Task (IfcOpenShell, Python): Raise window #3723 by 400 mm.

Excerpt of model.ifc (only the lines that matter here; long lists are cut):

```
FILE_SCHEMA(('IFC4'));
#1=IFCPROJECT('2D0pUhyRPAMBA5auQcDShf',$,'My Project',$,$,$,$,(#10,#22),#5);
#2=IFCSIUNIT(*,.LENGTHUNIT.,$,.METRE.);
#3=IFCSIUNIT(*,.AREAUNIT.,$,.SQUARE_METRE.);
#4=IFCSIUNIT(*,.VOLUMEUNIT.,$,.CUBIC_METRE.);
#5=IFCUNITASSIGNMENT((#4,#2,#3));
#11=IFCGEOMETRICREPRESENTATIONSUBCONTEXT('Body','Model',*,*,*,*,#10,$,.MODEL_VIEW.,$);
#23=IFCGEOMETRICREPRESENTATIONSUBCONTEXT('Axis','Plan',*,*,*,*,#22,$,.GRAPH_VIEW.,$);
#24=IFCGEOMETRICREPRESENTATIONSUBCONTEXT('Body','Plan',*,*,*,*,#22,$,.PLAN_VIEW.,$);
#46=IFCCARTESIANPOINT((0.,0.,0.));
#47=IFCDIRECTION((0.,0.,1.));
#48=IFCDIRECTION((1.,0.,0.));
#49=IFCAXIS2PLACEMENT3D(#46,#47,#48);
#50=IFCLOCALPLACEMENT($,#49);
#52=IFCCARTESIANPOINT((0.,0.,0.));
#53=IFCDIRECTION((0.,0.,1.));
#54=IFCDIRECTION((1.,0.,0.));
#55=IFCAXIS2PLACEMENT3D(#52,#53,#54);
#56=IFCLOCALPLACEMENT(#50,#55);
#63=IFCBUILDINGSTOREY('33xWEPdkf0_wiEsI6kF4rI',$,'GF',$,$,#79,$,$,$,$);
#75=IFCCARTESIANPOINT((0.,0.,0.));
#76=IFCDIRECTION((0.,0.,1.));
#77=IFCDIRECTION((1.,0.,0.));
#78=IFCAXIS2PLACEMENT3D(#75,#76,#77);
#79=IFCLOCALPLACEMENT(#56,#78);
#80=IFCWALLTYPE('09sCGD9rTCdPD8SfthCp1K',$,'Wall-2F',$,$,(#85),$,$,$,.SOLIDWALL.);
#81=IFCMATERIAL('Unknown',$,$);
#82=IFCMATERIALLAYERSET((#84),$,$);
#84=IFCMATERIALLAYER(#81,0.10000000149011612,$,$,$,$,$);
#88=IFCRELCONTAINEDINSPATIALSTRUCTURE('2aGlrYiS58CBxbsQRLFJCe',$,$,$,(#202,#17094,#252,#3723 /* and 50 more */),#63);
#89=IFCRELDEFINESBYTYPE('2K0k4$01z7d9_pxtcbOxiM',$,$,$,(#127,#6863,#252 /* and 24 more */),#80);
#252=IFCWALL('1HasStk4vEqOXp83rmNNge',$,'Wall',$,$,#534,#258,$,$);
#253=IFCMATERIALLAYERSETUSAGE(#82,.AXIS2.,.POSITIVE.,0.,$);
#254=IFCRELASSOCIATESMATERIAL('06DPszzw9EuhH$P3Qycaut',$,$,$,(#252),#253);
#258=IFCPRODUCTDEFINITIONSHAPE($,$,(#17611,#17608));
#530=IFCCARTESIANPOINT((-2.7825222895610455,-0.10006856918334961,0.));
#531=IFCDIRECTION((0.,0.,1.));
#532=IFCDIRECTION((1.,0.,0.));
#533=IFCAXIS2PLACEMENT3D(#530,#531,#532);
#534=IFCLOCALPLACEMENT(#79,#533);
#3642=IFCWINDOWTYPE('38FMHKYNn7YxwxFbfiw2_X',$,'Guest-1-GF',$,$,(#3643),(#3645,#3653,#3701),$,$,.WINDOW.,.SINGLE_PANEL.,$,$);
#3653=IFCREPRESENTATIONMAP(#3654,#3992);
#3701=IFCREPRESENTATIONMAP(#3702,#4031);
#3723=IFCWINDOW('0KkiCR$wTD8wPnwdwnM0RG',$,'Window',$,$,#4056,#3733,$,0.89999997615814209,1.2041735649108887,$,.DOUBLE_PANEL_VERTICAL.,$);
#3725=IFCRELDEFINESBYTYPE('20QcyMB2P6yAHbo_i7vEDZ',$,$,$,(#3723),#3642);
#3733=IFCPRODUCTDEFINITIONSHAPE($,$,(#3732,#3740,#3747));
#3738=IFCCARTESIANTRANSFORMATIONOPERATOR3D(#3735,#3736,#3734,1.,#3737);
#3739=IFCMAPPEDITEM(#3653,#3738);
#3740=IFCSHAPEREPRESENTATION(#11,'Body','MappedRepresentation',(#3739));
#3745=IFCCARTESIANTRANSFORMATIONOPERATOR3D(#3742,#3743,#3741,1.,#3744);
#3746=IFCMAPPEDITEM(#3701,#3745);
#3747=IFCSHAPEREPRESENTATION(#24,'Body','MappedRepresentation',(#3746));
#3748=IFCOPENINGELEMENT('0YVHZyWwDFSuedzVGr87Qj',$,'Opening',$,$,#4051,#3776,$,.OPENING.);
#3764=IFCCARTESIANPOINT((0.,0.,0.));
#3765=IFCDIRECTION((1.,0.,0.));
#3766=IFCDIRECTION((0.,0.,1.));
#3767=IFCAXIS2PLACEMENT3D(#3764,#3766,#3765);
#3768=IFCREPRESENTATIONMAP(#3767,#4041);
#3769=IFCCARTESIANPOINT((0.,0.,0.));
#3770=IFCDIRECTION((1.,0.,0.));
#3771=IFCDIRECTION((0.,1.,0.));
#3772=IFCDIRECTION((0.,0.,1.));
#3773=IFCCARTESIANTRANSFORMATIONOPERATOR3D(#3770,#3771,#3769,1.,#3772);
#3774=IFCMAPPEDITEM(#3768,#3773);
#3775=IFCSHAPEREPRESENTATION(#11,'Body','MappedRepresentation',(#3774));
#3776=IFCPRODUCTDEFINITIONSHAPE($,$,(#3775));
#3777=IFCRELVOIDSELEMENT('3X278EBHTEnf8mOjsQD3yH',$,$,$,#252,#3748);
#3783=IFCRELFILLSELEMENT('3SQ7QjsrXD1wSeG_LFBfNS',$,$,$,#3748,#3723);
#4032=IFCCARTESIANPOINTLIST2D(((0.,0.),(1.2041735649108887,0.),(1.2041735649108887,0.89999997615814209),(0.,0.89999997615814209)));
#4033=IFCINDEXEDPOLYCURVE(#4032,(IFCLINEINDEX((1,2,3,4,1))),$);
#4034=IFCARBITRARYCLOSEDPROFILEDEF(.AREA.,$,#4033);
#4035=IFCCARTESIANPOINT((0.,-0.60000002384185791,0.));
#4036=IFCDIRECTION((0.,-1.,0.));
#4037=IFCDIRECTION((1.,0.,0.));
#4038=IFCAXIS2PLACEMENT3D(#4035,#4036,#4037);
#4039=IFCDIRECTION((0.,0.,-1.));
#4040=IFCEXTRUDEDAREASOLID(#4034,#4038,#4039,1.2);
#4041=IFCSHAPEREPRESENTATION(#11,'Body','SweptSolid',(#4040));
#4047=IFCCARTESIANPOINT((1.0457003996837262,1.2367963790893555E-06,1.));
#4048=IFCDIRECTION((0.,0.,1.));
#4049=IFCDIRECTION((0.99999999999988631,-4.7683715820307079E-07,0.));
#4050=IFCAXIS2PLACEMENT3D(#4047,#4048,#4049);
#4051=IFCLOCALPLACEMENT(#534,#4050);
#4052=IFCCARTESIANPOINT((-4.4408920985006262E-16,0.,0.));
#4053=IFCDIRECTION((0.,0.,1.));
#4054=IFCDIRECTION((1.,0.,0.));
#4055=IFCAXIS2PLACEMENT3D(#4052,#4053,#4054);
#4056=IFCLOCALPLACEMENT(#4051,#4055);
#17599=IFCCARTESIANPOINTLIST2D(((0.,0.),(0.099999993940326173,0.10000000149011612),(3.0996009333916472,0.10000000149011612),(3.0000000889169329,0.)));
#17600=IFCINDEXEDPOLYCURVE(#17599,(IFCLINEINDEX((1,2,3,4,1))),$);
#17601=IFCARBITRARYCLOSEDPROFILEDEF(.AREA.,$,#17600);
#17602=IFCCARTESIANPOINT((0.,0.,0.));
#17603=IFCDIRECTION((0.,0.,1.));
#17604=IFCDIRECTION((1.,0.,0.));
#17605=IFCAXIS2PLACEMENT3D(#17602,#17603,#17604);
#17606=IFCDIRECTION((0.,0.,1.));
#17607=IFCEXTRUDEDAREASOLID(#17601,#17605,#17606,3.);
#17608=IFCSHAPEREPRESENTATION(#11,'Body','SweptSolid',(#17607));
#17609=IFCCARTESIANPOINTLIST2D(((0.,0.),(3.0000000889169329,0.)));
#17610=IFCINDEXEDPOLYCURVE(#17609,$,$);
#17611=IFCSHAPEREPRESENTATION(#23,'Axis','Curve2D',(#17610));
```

```python
import numpy as np
import ifcopenshell
import ifcopenshell.api.geometry
import ifcopenshell.util.placement
import ifcopenshell.util.unit

model = ifcopenshell.open("model.ifc")
unit_scale = ifcopenshell.util.unit.calculate_unit_scale(model)

window = model.by_id(3723)
opening = window.FillsVoids[0].RelatingOpeningElement
dz = 0.4 / unit_scale

shift = np.array([0.0, 0.0, dz])
# The window is placed relative to its opening, so it follows when the opening moves.
matrix = ifcopenshell.util.placement.get_local_placement(opening.ObjectPlacement)
matrix[:3, 3] += shift
ifcopenshell.api.geometry.edit_object_placement(
    model, product=opening, matrix=matrix, is_si=False, should_transform_children=True
)

print(f"moved by {dz * unit_scale:+.3f} m")

model.write("model-out.ifc")
```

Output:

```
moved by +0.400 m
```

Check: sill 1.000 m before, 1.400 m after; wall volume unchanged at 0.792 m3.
